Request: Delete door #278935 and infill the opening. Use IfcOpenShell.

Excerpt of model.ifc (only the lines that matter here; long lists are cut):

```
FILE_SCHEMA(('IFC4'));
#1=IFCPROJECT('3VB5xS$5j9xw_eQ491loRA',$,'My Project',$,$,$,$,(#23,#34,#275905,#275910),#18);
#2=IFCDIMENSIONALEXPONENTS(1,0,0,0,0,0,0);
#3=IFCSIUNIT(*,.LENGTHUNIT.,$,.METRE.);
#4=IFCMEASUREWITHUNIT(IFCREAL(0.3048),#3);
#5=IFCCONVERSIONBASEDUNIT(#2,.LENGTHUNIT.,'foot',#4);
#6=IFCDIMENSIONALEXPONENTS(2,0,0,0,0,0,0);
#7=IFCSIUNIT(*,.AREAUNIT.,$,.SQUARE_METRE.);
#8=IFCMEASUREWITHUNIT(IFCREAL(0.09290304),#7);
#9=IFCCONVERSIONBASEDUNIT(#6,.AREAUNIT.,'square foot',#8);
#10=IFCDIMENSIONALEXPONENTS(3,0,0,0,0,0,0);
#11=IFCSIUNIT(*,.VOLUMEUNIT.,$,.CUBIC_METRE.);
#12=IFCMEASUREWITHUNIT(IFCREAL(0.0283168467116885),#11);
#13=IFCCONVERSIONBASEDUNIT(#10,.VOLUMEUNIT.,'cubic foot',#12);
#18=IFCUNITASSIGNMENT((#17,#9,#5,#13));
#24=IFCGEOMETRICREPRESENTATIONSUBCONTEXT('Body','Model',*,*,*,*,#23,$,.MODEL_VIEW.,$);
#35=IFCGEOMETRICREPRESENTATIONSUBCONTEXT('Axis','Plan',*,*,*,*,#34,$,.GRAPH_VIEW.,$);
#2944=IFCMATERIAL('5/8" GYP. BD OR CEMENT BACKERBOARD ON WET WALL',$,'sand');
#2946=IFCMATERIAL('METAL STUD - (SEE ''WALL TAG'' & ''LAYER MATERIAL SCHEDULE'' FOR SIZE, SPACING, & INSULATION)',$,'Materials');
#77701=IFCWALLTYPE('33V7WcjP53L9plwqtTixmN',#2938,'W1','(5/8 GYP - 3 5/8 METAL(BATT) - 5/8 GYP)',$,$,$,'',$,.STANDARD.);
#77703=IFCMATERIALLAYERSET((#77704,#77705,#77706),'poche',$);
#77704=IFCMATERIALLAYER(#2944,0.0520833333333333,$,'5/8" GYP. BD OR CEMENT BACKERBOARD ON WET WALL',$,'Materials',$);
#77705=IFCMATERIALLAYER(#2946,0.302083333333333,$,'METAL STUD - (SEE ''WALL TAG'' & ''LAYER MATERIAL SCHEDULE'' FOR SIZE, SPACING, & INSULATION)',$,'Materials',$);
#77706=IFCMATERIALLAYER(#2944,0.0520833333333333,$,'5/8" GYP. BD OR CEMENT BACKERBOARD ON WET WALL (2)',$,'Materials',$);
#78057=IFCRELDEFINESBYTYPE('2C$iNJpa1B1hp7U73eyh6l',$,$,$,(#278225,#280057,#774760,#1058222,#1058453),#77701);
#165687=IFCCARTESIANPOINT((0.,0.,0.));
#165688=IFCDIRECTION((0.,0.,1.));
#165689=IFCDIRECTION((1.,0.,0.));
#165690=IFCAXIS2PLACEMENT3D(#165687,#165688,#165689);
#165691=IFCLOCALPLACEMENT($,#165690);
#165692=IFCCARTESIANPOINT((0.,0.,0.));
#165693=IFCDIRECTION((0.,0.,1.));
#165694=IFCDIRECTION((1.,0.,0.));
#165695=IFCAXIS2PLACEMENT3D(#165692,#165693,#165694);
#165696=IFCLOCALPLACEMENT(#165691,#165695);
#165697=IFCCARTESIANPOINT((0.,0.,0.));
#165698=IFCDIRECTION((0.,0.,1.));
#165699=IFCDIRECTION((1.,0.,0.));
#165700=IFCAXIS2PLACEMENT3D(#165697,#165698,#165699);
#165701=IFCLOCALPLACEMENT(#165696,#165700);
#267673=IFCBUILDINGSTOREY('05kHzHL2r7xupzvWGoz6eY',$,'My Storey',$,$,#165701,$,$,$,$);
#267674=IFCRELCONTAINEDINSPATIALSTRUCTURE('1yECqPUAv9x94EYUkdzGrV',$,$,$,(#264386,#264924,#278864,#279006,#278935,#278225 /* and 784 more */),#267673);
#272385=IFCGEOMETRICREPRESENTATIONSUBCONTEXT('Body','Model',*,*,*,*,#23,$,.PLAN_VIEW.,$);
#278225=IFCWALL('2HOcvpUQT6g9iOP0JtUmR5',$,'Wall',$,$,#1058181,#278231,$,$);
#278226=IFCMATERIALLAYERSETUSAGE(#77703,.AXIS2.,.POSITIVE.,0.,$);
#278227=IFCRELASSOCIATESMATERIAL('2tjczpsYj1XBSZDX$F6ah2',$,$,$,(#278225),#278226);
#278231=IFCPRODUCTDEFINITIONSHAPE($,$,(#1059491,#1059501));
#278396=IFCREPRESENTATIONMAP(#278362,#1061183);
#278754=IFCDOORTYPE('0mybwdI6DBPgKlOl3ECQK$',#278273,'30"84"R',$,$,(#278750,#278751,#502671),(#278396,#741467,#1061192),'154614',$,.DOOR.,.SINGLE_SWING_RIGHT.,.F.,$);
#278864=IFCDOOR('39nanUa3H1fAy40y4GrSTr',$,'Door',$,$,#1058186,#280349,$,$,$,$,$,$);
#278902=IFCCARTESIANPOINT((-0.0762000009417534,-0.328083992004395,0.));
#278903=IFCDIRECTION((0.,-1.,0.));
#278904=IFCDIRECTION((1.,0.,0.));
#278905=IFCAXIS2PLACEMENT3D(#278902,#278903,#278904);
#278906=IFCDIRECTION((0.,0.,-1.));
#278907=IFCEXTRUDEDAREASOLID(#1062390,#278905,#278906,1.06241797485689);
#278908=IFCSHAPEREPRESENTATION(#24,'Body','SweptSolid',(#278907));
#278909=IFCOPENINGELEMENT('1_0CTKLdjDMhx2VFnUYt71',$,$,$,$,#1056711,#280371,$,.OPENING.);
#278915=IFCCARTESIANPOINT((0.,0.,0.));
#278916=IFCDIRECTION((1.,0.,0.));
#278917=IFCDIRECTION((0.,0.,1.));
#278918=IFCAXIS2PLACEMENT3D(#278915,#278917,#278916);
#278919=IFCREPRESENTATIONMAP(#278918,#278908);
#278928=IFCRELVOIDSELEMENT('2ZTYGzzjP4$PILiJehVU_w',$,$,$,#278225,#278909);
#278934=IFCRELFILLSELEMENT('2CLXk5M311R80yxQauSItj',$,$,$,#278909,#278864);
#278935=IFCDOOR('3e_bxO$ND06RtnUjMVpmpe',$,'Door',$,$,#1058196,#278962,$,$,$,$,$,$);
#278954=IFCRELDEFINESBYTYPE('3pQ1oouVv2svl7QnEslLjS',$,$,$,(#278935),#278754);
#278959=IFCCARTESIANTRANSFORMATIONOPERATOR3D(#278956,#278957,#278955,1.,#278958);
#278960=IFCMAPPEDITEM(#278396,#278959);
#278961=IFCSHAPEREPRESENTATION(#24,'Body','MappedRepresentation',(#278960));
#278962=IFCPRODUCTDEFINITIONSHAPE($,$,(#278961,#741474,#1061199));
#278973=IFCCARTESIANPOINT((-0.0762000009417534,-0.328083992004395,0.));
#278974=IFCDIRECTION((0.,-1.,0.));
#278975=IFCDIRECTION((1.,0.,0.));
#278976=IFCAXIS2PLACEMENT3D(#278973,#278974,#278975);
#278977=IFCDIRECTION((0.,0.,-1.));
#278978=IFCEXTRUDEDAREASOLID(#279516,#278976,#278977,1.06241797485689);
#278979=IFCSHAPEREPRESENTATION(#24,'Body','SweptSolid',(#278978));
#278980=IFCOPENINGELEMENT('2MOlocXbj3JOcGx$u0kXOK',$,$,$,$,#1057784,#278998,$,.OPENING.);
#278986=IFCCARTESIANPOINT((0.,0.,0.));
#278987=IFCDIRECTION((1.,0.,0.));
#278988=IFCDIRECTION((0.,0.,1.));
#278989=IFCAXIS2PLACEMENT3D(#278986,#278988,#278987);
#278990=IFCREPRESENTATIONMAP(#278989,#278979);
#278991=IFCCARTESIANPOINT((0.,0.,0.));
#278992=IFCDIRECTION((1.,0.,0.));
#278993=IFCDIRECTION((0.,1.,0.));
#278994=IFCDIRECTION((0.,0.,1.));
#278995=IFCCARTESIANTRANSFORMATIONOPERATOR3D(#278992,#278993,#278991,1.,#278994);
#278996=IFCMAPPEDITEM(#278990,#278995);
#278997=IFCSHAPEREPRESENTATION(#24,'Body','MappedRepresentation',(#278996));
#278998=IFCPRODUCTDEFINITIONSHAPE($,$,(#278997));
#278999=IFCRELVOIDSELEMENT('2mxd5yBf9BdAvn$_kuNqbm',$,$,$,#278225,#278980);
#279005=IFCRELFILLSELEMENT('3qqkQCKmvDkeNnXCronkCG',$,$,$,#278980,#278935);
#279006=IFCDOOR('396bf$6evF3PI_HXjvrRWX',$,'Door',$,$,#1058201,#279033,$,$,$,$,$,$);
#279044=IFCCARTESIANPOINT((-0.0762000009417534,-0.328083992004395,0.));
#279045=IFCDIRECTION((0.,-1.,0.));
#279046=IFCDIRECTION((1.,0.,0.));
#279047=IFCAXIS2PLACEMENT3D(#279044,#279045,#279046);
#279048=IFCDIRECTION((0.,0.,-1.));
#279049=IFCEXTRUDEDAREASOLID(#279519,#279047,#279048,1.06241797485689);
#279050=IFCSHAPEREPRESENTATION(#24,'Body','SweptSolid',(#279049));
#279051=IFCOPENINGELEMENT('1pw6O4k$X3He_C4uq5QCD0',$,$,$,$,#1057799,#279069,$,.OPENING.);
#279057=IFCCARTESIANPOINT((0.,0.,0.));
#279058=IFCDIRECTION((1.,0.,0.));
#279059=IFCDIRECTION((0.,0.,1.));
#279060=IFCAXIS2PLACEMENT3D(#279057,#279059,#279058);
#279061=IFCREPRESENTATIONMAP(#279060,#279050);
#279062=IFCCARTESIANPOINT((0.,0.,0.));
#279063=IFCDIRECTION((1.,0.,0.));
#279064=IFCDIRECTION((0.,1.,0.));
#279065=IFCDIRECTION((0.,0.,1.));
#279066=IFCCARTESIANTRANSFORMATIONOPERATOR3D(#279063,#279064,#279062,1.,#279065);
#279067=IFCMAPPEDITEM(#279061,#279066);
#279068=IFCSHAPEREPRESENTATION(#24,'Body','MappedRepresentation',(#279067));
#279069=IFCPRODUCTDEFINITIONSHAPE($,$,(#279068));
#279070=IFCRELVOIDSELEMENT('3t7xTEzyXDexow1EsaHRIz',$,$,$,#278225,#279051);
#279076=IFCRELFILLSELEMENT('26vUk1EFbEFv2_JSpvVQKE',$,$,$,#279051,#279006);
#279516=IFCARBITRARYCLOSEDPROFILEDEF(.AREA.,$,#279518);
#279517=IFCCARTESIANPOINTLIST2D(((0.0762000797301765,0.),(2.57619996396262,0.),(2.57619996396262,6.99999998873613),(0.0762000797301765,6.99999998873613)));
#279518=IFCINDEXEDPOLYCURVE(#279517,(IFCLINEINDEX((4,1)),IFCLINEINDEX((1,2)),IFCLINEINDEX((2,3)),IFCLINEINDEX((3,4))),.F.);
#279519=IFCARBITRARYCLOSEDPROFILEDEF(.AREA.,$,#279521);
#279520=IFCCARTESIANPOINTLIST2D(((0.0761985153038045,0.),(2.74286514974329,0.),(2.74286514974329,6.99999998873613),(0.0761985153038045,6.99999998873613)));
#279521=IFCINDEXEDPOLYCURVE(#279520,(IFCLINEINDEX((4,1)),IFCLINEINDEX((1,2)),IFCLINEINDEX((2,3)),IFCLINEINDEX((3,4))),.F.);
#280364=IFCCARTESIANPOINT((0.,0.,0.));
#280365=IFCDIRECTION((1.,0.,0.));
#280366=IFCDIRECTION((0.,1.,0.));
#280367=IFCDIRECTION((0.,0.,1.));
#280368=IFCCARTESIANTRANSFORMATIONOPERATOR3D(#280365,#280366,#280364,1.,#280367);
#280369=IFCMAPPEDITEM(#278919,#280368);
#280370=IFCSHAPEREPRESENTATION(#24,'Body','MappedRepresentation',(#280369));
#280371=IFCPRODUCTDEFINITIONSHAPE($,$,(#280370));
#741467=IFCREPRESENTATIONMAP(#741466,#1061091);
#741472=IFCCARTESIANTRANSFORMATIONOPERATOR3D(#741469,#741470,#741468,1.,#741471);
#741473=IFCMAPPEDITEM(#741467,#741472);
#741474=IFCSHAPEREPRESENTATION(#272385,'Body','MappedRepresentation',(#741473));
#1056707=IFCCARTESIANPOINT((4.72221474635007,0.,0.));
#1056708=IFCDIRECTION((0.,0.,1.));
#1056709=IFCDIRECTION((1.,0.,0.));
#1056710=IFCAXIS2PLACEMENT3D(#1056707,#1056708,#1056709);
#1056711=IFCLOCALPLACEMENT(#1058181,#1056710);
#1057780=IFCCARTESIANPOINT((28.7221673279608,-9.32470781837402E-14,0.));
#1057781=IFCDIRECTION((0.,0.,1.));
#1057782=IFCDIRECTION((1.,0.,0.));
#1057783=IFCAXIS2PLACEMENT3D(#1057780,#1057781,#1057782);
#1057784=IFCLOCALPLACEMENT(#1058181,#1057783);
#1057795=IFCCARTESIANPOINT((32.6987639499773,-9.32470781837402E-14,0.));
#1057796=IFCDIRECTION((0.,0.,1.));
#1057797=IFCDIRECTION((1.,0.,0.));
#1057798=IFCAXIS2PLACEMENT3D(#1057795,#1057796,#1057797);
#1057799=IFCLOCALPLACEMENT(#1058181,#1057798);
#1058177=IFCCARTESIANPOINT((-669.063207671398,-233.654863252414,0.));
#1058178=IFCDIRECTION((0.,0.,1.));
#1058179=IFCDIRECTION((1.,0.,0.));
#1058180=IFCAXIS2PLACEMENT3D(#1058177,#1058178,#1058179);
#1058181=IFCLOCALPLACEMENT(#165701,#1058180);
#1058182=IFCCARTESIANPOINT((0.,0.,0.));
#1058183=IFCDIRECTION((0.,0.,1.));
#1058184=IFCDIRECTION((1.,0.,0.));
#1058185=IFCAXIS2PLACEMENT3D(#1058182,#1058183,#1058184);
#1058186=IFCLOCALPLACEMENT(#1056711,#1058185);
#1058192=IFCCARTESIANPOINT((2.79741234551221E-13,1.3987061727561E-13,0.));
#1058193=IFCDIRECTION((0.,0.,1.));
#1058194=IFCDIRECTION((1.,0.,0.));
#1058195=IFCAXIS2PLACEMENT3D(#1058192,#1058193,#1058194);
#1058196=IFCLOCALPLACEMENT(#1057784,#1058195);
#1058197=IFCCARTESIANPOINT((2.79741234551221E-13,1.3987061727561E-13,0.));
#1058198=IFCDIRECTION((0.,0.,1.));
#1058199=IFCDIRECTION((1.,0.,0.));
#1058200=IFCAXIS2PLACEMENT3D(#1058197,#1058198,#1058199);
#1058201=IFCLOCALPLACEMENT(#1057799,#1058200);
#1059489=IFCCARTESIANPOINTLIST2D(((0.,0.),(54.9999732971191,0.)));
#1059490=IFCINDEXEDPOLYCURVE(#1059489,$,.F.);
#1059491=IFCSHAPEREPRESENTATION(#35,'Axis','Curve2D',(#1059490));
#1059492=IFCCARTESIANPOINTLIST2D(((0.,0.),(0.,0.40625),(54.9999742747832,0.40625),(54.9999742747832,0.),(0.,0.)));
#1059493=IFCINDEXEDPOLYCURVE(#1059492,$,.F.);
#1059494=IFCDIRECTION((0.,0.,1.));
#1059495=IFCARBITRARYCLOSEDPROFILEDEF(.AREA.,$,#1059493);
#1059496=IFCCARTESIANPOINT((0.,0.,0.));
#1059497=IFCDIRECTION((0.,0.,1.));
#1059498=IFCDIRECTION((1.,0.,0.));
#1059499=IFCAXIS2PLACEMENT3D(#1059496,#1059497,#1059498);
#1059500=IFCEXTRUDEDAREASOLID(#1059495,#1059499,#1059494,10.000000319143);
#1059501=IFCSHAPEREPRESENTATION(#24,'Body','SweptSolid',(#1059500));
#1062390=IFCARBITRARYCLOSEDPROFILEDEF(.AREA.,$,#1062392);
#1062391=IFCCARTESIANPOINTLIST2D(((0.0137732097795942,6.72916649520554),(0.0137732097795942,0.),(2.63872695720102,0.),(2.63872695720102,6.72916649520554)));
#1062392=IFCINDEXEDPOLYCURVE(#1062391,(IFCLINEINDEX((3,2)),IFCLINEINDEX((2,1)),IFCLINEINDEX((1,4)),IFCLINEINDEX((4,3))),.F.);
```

```python
import ifcopenshell
import ifcopenshell.api.feature
import ifcopenshell.api.root
import ifcopenshell.geom
import ifcopenshell.util.shape

model = ifcopenshell.open("model.ifc")
settings = ifcopenshell.geom.settings()


def volume(element):
    """Net volume in cubic metres, openings subtracted."""
    shape = ifcopenshell.geom.create_shape(settings, element)
    return ifcopenshell.util.shape.get_volume(shape.geometry)


door = model.by_id(278935)
opening = door.FillsVoids[0].RelatingOpeningElement
wall = opening.VoidsElements[0].RelatingBuildingElement
before = volume(wall)

ifcopenshell.api.root.remove_product(model, product=door)
ifcopenshell.api.feature.remove_feature(model, feature=opening)

after = volume(wall)

print(f"wall volume {before:.3f} -> {after:.3f} m3")

model.write("model_v2.ifc")
```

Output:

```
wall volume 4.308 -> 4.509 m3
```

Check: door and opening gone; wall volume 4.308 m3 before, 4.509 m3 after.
